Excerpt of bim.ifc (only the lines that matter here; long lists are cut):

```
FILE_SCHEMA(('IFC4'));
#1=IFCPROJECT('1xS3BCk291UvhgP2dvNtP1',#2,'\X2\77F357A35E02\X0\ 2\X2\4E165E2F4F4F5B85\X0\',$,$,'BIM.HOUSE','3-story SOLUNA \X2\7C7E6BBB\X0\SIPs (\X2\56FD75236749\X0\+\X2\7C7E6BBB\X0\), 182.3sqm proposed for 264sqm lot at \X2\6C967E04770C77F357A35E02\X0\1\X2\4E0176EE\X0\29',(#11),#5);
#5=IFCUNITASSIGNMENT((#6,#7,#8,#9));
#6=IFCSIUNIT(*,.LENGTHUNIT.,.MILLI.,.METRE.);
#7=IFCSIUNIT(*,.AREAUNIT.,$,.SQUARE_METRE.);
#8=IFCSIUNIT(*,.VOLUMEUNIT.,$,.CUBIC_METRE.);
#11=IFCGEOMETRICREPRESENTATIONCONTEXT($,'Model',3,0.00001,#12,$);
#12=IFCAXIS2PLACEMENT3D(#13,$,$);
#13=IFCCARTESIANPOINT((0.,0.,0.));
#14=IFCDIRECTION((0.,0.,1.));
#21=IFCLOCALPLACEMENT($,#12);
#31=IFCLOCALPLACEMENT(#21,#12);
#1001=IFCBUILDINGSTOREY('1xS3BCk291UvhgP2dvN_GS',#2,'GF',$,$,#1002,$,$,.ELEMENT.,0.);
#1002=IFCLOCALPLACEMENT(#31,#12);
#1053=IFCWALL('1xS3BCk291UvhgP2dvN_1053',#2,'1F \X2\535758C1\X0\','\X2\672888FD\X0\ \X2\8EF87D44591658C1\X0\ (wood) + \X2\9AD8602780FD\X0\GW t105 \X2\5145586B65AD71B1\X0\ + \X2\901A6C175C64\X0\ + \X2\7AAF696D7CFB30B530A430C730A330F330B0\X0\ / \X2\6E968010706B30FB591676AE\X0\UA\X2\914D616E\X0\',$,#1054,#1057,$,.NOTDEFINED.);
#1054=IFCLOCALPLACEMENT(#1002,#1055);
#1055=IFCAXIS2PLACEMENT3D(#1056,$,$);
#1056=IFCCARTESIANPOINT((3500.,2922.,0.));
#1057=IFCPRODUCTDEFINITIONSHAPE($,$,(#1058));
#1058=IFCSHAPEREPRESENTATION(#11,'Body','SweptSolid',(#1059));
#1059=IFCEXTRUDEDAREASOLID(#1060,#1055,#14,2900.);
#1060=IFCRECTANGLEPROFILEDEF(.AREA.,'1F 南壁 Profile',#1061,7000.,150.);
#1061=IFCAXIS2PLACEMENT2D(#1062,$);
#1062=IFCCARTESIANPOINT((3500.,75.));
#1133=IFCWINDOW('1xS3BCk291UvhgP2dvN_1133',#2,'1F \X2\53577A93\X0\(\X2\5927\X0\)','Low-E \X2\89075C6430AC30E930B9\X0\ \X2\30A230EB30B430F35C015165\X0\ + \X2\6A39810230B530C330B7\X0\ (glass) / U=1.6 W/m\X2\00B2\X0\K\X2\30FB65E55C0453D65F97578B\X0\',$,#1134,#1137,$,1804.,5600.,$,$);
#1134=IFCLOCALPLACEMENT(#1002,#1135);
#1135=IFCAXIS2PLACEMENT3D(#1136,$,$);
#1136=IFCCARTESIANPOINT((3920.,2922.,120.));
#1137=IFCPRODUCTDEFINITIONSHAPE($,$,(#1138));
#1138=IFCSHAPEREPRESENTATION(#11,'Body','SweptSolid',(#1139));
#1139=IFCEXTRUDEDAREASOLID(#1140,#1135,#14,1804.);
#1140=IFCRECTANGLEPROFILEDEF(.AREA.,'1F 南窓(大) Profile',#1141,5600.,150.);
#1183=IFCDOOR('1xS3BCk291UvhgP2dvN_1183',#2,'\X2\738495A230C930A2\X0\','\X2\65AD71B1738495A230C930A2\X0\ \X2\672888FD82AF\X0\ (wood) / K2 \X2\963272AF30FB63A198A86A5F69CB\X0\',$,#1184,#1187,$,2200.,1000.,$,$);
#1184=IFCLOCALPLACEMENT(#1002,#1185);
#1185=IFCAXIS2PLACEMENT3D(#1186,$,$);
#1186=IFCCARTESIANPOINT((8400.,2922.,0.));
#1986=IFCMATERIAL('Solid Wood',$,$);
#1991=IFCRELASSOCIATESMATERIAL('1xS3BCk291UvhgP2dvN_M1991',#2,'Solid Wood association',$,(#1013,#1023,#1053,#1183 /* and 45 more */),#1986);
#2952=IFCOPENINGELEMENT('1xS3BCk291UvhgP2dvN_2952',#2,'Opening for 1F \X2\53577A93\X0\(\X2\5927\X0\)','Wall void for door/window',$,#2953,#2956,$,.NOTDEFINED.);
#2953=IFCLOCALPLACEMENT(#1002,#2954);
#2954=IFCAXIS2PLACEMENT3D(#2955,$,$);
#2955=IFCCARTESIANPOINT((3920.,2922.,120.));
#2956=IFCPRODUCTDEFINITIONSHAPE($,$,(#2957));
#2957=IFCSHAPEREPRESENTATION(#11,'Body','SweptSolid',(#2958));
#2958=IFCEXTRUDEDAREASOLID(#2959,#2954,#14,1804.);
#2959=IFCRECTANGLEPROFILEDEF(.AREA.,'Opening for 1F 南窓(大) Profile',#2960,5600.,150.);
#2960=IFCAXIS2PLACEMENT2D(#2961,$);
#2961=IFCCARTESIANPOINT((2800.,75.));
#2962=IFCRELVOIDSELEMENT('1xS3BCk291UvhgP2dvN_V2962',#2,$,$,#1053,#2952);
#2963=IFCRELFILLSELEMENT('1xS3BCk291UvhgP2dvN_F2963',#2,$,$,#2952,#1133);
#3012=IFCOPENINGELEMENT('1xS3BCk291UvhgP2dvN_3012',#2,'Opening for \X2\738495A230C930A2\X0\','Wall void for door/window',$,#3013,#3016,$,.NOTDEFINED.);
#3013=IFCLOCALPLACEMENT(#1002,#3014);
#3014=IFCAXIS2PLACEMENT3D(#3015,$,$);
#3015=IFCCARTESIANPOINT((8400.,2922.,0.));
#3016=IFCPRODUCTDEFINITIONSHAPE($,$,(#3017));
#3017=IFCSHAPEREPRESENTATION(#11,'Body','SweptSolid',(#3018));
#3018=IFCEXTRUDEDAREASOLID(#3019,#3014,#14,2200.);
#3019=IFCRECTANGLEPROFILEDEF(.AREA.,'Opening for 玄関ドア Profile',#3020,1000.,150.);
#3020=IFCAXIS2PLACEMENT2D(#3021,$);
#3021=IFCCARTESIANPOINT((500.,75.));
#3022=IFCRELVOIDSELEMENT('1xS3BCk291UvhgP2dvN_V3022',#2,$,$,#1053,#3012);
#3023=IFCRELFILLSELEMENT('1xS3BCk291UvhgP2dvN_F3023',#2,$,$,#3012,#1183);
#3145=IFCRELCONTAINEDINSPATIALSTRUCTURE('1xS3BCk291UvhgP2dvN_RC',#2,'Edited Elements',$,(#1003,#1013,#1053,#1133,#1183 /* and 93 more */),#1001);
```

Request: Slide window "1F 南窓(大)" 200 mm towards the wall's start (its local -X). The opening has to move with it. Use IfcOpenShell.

```python
import ifcopenshell
import ifcopenshell.api.geometry
import ifcopenshell.util.placement
import ifcopenshell.util.unit

model = ifcopenshell.open("bim.ifc")
unit_scale = ifcopenshell.util.unit.calculate_unit_scale(model)

window = model.by_guid("1xS3BCk291UvhgP2dvN_1133")
opening = window.FillsVoids[0].RelatingOpeningElement
wall = opening.VoidsElements[0].RelatingBuildingElement

wall_matrix = ifcopenshell.util.placement.get_local_placement(wall.ObjectPlacement)
shift = wall_matrix[:3, 0] * -0.2 / unit_scale
before = ifcopenshell.util.placement.get_local_placement(window.ObjectPlacement)[:3, 3].copy()

# The window is not placed relative to its opening, so move both.
for product in (opening, window):
    matrix = ifcopenshell.util.placement.get_local_placement(product.ObjectPlacement)
    matrix[:3, 3] += shift
    ifcopenshell.api.geometry.edit_object_placement(model, product=product, matrix=matrix, is_si=False)

after = ifcopenshell.util.placement.get_local_placement(window.ObjectPlacement)[:3, 3]
print("window moved by", (after - before).round(3) + 0.0)

model.write("bim_v2.ifc")
```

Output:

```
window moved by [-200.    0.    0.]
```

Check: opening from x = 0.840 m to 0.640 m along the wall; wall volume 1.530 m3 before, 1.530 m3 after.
